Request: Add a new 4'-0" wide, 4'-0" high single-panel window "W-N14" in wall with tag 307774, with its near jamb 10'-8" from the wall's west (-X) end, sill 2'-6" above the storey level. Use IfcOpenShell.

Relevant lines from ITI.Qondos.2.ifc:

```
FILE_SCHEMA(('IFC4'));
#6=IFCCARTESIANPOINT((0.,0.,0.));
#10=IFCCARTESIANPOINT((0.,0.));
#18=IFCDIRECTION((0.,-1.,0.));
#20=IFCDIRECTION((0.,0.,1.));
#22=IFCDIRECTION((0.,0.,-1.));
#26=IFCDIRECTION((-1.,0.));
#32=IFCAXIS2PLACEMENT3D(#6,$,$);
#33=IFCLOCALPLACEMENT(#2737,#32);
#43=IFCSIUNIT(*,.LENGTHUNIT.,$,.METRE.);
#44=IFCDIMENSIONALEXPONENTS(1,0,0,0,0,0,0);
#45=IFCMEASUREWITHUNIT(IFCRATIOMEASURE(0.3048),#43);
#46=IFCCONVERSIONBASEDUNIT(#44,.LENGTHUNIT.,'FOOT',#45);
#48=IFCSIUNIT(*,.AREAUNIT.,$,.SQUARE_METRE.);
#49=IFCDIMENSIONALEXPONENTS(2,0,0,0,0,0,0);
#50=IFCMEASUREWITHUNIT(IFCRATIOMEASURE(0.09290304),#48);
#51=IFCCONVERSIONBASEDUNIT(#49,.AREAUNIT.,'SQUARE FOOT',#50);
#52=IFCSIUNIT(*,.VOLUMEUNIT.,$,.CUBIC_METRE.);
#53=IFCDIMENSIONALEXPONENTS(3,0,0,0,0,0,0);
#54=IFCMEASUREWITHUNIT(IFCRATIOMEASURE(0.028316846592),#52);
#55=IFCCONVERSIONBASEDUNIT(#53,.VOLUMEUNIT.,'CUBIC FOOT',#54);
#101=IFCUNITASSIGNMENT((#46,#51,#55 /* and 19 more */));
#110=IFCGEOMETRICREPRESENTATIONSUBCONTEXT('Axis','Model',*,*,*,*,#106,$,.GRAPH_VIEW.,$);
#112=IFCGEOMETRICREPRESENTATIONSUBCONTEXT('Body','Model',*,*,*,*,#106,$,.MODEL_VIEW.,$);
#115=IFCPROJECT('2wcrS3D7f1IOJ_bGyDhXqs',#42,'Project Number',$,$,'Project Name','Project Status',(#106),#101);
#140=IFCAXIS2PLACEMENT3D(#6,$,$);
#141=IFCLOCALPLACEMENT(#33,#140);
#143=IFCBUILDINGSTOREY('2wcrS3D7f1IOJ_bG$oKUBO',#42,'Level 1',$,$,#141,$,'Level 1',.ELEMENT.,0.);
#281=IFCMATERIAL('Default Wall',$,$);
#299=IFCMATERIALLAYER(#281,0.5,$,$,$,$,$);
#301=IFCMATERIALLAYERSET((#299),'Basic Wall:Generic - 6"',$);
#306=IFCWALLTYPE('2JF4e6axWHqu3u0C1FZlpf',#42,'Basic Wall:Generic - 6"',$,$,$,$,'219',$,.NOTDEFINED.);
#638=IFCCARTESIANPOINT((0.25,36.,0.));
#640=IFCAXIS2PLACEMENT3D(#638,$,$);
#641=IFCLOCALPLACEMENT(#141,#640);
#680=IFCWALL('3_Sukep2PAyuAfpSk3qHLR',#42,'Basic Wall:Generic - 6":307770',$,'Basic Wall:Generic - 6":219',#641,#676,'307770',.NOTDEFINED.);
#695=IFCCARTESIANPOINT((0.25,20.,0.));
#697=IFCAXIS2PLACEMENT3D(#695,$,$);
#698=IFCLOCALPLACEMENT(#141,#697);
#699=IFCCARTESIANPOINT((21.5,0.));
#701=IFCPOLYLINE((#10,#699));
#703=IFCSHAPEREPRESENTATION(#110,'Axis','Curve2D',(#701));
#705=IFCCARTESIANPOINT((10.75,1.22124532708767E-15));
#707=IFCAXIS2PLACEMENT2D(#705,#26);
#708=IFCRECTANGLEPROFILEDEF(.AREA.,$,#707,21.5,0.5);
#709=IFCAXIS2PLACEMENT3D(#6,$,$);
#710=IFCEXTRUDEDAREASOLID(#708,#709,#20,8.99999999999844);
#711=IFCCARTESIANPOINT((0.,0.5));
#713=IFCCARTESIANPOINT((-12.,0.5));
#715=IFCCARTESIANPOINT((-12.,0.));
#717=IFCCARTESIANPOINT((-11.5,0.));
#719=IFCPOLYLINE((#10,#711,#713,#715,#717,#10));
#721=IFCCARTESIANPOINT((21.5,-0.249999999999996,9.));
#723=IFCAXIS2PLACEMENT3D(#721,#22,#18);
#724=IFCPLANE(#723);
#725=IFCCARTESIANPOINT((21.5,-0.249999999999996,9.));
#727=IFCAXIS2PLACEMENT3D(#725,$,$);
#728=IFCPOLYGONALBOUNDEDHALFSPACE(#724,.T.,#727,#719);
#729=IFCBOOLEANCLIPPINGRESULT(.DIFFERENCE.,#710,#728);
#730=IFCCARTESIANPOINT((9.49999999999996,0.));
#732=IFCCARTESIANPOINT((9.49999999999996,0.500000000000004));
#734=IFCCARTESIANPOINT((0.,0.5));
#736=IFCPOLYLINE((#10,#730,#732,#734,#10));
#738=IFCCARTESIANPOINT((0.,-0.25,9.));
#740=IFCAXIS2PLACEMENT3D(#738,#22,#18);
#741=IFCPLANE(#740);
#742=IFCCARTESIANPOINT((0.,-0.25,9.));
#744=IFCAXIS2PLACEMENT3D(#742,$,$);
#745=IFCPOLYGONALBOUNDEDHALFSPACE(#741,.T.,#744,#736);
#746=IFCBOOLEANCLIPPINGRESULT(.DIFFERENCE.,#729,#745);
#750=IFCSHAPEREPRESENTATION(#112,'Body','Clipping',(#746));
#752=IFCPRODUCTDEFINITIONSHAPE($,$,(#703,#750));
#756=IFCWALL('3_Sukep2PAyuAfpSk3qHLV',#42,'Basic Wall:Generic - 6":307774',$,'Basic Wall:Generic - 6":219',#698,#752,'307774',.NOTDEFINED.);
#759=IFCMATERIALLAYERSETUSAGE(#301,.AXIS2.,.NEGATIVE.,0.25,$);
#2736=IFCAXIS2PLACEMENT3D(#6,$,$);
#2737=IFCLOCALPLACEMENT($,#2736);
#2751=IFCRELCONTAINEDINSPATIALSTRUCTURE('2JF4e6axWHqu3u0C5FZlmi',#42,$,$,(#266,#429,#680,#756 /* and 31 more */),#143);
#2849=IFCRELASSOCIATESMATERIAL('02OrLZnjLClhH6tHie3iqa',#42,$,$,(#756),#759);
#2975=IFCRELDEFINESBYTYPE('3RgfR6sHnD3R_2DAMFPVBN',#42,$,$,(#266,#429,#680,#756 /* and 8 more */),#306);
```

```python
import numpy as np
import ifcopenshell
import ifcopenshell.api.feature
import ifcopenshell.api.geometry
import ifcopenshell.api.root
import ifcopenshell.api.spatial
import ifcopenshell.geom
import ifcopenshell.util.element
import ifcopenshell.util.placement
import ifcopenshell.util.representation
import ifcopenshell.util.shape
import ifcopenshell.util.unit

model = ifcopenshell.open("ITI.Qondos.2.ifc")
unit_scale = ifcopenshell.util.unit.calculate_unit_scale(model)
settings = ifcopenshell.geom.settings()


def volume(element):
    """Net volume in cubic metres, openings subtracted."""
    shape = ifcopenshell.geom.create_shape(settings, element)
    return ifcopenshell.util.shape.get_volume(shape.geometry)


wall = model.by_guid("3_Sukep2PAyuAfpSk3qHLV")
storey = ifcopenshell.util.element.get_container(wall, ifc_class="IfcBuildingStorey")
context = ifcopenshell.util.representation.get_context(model, "Model", "Body", "MODEL_VIEW")
before = volume(wall)

width, height, from_end, sill = 1.2192, 1.2192, 3.2512, 0.762  # metres

# The wall runs along its own X axis, and the end named is its -X end.
wall_shape = ifcopenshell.geom.create_shape(settings, wall)
x, y, z = ifcopenshell.util.shape.get_vertices(wall_shape.geometry).T
start = x.min() + from_end
face, thickness = float(y.min()), float(y.max() - y.min())
wall_matrix = ifcopenshell.util.placement.get_local_placement(wall.ObjectPlacement)
level = ifcopenshell.util.placement.get_local_placement(storey.ObjectPlacement)[2, 3]


def in_wall(x, y):
    """Placement at x, y metres in the wall's axes, at sill height."""
    matrix = wall_matrix.copy()
    matrix[:, 3] = wall_matrix @ np.array([x / unit_scale, y / unit_scale, 0.0, 1.0])
    matrix[2, 3] = level + sill / unit_scale
    return matrix


# Opening: a box that overshoots both wall faces by 50 mm.
opening = ifcopenshell.api.root.create_entity(model, ifc_class="IfcOpeningElement", predefined_type="OPENING")
box = ifcopenshell.api.geometry.add_wall_representation(
    model, context=context, length=width, height=height, thickness=thickness + 0.1
)
ifcopenshell.api.geometry.assign_representation(model, product=opening, representation=box)
ifcopenshell.api.geometry.edit_object_placement(model, product=opening, matrix=in_wall(start, face - 0.05), is_si=False)
ifcopenshell.api.feature.add_feature(model, feature=opening, element=wall)

window = ifcopenshell.api.root.create_entity(model, ifc_class="IfcWindow", name="W-N14", predefined_type="WINDOW")
window.OverallWidth, window.OverallHeight = width / unit_scale, height / unit_scale
window.PartitioningType = "SINGLE_PANEL"
body = ifcopenshell.api.geometry.add_window_representation(
    model,
    context=context,
    overall_width=window.OverallWidth,
    overall_height=window.OverallHeight,
    partition_type="SINGLE_PANEL",
)
ifcopenshell.api.geometry.assign_representation(model, product=window, representation=body)
ifcopenshell.api.spatial.assign_container(model, products=[window], relating_structure=storey)
ifcopenshell.api.feature.add_filling(model, opening=opening, element=window)

# Centre the window in the wall's thickness.
ifcopenshell.api.geometry.edit_object_placement(model, product=window, matrix=in_wall(start, face), is_si=False)
window_shape = ifcopenshell.geom.create_shape(settings, window)
depth = ifcopenshell.util.shape.get_vertices(window_shape.geometry)[:, 1]
offset = face + thickness / 2 - (depth.min() + depth.max()) / 2
ifcopenshell.api.geometry.edit_object_placement(model, product=window, matrix=in_wall(start, offset), is_si=False)

after = volume(wall)

print(f"wall volume {before:.3f} -> {after:.3f} m3")

model.write("ITI.Qondos.2-out.ifc")
```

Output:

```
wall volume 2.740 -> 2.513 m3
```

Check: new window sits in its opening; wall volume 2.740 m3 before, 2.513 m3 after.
